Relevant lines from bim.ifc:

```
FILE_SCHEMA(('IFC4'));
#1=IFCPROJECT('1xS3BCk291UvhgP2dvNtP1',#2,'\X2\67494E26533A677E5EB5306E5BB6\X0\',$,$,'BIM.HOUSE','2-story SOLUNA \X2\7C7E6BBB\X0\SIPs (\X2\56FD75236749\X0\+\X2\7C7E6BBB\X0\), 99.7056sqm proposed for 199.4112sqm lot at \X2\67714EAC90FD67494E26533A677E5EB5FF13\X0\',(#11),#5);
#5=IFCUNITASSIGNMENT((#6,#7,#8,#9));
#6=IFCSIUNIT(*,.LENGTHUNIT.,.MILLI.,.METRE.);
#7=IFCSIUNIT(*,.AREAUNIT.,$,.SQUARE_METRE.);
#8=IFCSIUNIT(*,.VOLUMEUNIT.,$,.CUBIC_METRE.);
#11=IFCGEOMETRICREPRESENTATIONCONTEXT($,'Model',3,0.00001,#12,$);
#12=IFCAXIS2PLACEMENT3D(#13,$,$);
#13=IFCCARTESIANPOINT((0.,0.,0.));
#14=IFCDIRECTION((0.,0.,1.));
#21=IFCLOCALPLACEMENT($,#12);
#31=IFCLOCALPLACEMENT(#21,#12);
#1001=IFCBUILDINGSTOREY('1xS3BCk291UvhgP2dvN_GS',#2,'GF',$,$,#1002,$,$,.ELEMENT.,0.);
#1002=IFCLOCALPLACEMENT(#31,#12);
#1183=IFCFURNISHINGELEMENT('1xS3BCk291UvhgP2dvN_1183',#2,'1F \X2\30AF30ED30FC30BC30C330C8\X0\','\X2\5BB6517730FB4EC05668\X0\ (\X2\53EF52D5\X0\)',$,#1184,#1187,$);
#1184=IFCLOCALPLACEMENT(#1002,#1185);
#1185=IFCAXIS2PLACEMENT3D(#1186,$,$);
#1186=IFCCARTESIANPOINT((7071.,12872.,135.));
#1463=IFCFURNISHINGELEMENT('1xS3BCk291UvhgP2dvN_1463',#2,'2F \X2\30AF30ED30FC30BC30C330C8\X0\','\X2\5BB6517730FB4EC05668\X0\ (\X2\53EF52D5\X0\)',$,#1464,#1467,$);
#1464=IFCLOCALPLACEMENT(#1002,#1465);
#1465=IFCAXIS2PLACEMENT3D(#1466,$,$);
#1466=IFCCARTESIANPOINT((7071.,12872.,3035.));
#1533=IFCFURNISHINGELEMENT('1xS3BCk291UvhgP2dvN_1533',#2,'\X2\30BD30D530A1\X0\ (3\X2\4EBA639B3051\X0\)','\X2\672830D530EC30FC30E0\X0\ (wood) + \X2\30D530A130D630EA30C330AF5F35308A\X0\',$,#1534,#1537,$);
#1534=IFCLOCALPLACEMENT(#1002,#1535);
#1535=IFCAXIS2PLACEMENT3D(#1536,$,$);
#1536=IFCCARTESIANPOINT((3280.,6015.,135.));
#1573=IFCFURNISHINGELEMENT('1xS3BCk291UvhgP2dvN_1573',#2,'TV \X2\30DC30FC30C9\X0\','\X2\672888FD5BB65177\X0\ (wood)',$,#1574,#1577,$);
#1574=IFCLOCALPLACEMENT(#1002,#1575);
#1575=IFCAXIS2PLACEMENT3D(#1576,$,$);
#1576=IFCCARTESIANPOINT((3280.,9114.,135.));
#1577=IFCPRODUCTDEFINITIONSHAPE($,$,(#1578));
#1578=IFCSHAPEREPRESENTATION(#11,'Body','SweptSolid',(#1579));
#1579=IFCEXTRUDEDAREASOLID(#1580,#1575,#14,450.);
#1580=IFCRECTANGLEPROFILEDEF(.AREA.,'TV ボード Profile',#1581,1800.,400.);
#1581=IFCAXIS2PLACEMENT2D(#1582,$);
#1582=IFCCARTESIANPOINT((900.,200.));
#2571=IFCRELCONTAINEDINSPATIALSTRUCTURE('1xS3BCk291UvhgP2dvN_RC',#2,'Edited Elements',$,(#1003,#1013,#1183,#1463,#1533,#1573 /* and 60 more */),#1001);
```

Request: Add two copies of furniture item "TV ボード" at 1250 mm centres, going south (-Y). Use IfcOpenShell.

```python
import numpy as np
import ifcopenshell
import ifcopenshell.api.geometry
import ifcopenshell.api.root
import ifcopenshell.util.element
import ifcopenshell.util.placement
import ifcopenshell.util.unit

model = ifcopenshell.open("bim.ifc")
unit_scale = ifcopenshell.util.unit.calculate_unit_scale(model)


def reuse_history(source, copy):
    """copy_class also copies each property set's owner history, people and application; keep the originals."""
    for rel in copy.IsDefinedBy:
        if rel.is_a("IfcRelDefinesByProperties") and (history := rel.RelatingPropertyDefinition.OwnerHistory):
            rel.RelatingPropertyDefinition.OwnerHistory = source.OwnerHistory
            ifcopenshell.util.element.remove_deep2(model, history)


source = model.by_guid("1xS3BCk291UvhgP2dvN_1573")
base = ifcopenshell.util.placement.get_local_placement(source.ObjectPlacement)
step = np.array([0.0, -1.0, 0.0]) * 1.25 / unit_scale

for i in range(1, 3):
    copy = ifcopenshell.api.root.copy_class(model, product=source)
    copy.Representation = ifcopenshell.util.element.copy_deep(
        model, source.Representation, exclude=["IfcGeometricRepresentationContext", "IfcRepresentationMap"]
    )
    reuse_history(source, copy)
    matrix = base.copy()
    matrix[:3, 3] += i * step
    print("added at", matrix[:3, 3].round(3) + 0.0)
    ifcopenshell.api.geometry.edit_object_placement(model, product=copy, matrix=matrix, is_si=False)

model.write("bim_v2.ifc")
```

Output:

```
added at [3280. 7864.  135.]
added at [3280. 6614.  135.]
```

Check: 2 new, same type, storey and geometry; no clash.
